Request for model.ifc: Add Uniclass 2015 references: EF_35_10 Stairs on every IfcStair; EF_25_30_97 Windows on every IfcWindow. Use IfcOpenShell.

First a look at what the model holds.

```python
import ifcopenshell

model = ifcopenshell.open("model.ifc")
print(model.schema)
print("classifications:", [c.Name for c in model.by_type("IfcClassification")])
for ifc_class in ("IfcDoor", "IfcRoof", "IfcStair", "IfcWall", "IfcWindow"):
    print(ifc_class, len(model.by_type(ifc_class)))
```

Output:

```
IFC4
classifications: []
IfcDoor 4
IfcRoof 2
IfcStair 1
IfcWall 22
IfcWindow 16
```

```python
import ifcopenshell
import ifcopenshell.api.classification

model = ifcopenshell.open("model.ifc")

system = ifcopenshell.api.classification.add_classification(model, classification="Uniclass 2015")

codes = {
    "IfcStair": ("EF_35_10", "Stairs"),
    "IfcWindow": ("EF_25_30_97", "Windows"),
}
for ifc_class, (code, name) in codes.items():
    products = model.by_type(ifc_class)
    ifcopenshell.api.classification.add_reference(
        model, products=products, classification=system, identification=code, name=name
    )
    print(code, len(products))

model.write("model_updated.ifc")
```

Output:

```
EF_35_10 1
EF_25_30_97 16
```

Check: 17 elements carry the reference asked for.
